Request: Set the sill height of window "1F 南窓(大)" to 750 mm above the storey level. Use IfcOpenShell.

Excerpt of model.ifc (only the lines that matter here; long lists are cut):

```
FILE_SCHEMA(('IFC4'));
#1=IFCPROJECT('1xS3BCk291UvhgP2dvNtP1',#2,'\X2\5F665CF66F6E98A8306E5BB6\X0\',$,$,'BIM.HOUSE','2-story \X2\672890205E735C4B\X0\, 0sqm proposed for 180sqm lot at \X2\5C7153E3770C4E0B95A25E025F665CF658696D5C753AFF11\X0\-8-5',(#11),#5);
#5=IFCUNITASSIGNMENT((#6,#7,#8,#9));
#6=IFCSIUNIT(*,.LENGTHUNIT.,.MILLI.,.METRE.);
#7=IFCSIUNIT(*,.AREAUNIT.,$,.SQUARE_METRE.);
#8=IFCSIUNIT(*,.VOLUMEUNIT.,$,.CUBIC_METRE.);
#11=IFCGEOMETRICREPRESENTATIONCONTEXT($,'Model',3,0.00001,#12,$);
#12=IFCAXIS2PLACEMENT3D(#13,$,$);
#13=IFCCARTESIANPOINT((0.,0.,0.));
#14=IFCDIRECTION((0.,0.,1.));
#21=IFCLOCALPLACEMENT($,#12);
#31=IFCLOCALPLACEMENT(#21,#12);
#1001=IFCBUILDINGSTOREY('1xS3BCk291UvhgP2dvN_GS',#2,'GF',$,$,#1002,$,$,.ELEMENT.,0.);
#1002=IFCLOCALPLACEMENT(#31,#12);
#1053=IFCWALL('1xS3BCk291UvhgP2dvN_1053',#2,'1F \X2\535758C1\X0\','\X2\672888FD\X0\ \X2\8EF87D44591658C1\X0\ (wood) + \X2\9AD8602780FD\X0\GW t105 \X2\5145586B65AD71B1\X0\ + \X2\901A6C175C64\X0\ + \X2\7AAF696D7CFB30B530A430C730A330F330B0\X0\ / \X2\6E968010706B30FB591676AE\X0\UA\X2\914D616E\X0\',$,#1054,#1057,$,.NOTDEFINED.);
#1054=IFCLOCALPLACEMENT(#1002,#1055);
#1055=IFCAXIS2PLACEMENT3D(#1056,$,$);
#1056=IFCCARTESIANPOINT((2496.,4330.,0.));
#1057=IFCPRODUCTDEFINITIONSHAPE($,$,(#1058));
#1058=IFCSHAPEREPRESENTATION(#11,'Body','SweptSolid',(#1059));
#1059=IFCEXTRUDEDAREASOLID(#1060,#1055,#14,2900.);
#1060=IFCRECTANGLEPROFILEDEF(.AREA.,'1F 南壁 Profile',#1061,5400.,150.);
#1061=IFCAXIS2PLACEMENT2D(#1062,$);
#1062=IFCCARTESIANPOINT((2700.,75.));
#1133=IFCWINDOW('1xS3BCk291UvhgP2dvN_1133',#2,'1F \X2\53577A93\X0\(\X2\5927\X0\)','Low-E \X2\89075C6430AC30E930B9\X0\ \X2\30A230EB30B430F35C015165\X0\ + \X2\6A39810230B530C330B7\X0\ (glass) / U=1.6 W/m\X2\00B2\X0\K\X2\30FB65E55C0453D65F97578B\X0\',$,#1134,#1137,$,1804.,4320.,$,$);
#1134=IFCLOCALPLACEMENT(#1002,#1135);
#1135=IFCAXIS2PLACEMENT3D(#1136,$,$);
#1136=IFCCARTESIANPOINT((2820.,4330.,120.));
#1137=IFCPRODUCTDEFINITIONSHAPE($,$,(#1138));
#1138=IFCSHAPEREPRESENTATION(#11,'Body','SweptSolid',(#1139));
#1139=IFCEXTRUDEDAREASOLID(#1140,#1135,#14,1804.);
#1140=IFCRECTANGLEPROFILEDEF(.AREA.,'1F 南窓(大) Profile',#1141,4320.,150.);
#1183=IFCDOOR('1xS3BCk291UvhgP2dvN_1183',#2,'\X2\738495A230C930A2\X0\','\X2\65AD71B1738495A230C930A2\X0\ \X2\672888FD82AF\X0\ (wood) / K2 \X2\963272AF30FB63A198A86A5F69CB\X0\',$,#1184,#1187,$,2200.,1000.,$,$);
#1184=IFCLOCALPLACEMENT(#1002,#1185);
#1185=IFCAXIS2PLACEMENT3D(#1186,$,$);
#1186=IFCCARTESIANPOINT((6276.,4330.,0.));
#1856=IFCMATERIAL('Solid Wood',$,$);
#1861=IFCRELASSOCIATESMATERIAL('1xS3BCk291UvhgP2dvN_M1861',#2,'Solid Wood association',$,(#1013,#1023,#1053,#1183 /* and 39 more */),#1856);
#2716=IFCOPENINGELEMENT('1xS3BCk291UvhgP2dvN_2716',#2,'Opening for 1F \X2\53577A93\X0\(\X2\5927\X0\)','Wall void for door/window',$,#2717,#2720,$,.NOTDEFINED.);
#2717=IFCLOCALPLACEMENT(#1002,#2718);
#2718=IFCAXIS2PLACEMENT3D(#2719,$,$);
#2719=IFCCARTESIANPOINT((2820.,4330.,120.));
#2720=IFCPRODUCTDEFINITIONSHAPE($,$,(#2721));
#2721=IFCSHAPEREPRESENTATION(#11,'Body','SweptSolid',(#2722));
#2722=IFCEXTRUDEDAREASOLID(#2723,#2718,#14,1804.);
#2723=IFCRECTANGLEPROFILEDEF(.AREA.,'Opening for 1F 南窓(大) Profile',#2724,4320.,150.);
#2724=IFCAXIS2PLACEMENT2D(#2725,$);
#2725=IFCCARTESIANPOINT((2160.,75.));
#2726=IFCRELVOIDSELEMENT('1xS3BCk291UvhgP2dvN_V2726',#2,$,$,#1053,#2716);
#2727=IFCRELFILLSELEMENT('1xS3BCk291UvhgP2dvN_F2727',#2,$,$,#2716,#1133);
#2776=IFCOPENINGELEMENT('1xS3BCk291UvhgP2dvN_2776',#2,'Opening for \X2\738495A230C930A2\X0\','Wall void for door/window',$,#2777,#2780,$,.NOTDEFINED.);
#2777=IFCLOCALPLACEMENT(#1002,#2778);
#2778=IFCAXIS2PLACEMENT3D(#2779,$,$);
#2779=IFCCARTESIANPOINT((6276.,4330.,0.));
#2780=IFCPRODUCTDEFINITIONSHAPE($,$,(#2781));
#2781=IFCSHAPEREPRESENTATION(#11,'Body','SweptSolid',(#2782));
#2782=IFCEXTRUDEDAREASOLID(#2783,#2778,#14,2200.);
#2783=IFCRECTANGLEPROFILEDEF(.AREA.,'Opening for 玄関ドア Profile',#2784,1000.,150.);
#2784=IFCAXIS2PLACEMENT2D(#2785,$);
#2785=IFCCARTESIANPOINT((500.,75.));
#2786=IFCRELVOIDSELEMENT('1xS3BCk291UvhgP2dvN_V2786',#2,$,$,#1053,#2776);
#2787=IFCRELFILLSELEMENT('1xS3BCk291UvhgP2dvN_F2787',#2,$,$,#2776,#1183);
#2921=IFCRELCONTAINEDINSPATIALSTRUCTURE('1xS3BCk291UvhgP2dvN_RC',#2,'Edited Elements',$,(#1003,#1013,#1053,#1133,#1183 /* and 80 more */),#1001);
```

```python
import numpy as np
import ifcopenshell
import ifcopenshell.api.geometry
import ifcopenshell.geom
import ifcopenshell.util.element
import ifcopenshell.util.placement
import ifcopenshell.util.shape
import ifcopenshell.util.unit

model = ifcopenshell.open("model.ifc")
unit_scale = ifcopenshell.util.unit.calculate_unit_scale(model)

window = model.by_guid("1xS3BCk291UvhgP2dvN_1133")
opening = window.FillsVoids[0].RelatingOpeningElement
storey = ifcopenshell.util.element.get_container(window, ifc_class="IfcBuildingStorey")
level = ifcopenshell.util.placement.get_local_placement(storey.ObjectPlacement)[2, 3]

# The opening's origin need not be at the sill, so measure its lowest point.
shape = ifcopenshell.geom.create_shape(ifcopenshell.geom.settings(), opening)
bottom = ifcopenshell.util.shape.get_shape_bottom_elevation(shape, shape.geometry) / unit_scale
dz = level + 750.0 - bottom

shift = np.array([0.0, 0.0, dz])
# The window is not placed relative to its opening, so move both.
for product in (opening, window):
    matrix = ifcopenshell.util.placement.get_local_placement(product.ObjectPlacement)
    matrix[:3, 3] += shift
    ifcopenshell.api.geometry.edit_object_placement(model, product=product, matrix=matrix, is_si=False)

print(f"moved by {dz * unit_scale:+.3f} m")

model.write("model_updated.ifc")
```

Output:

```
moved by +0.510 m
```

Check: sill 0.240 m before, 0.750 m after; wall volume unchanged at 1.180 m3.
